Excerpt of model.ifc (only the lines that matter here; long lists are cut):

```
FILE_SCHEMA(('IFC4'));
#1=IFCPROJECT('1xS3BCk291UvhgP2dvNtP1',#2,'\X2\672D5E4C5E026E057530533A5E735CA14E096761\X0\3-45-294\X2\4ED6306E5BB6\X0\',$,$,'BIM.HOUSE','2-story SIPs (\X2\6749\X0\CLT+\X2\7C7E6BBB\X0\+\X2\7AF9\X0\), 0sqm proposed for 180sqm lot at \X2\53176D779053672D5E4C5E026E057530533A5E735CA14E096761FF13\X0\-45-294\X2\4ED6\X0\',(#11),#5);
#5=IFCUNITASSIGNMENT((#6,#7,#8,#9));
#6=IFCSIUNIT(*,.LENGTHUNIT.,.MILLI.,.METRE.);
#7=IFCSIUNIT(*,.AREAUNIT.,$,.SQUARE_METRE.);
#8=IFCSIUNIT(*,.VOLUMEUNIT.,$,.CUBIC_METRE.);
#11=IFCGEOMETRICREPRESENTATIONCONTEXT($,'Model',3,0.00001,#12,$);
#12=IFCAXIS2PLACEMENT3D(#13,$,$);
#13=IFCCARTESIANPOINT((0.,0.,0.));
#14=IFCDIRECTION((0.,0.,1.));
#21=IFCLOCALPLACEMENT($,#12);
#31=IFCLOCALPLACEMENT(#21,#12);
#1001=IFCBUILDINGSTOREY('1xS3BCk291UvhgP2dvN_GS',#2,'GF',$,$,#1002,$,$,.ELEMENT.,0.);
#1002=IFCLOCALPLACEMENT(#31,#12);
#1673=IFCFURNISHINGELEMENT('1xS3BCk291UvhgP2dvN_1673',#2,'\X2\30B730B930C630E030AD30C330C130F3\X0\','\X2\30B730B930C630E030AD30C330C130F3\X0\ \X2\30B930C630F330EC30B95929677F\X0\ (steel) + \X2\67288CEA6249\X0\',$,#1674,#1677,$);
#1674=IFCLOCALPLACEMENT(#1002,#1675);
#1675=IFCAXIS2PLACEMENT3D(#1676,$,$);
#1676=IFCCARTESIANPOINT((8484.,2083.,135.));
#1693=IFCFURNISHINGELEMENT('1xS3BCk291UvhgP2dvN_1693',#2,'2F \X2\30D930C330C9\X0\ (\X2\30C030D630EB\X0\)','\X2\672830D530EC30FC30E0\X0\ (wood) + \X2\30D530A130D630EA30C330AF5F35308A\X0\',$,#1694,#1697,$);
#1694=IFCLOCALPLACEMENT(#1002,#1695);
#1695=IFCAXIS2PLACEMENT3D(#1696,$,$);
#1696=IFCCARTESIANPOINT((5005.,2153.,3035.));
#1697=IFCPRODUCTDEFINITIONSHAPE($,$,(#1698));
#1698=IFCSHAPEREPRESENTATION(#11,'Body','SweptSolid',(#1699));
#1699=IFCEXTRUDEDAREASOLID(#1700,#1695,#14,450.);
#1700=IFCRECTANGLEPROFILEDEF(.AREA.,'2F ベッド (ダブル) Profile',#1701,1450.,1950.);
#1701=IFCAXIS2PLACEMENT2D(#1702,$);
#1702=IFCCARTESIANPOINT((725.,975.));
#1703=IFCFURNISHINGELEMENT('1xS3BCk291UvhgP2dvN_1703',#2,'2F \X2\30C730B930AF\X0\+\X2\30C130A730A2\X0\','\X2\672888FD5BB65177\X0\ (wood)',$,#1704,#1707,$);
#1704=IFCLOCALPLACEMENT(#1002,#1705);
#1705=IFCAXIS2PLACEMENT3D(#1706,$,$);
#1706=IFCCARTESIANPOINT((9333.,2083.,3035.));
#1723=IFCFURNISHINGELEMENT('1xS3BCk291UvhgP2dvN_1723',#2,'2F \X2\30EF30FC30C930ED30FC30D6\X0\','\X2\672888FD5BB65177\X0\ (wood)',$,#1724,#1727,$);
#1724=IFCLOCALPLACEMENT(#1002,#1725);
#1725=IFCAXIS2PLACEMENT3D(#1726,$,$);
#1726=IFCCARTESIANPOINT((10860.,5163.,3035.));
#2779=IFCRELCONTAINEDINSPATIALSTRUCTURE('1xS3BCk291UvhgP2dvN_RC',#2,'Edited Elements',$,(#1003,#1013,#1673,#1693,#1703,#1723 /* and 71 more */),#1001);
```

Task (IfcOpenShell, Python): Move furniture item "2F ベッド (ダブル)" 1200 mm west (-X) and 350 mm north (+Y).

```python
import ifcopenshell
import ifcopenshell.api.geometry
import ifcopenshell.util.placement

model = ifcopenshell.open("model.ifc")

item = model.by_id(1693)
matrix = ifcopenshell.util.placement.get_local_placement(item.ObjectPlacement)
matrix[0, 3] -= 1200.0
matrix[1, 3] += 350.0
ifcopenshell.api.geometry.edit_object_placement(model, product=item, matrix=matrix, is_si=False)

print(ifcopenshell.util.placement.get_local_placement(item.ObjectPlacement).round(3) + 0.0)

model.write("model-out.ifc")
```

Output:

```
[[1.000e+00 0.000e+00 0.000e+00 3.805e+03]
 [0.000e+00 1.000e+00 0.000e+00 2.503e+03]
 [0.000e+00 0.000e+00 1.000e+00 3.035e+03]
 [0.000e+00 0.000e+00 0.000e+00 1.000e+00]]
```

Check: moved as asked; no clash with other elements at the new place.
